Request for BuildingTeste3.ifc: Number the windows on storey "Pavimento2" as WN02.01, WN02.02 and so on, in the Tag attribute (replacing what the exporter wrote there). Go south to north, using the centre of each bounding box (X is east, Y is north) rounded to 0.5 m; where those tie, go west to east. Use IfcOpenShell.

First a look at what the model holds.

```python
import ifcopenshell
import ifcopenshell.util.element
import ifcopenshell.util.placement

model = ifcopenshell.open("BuildingTeste3.ifc")
print(model.schema)
storey = next(s for s in model.by_type("IfcBuildingStorey") if s.Name == "Pavimento2")
windows = [e for e in ifcopenshell.util.element.get_decomposition(storey) if e.is_a("IfcWindow")]
for e in sorted(windows, key=lambda e: e.id()):
    origin = ifcopenshell.util.placement.get_local_placement(e.ObjectPlacement)[:3, 3]
    print(e.id(), e.Tag, e.Name, origin.round(2) + 0.0, sep=" | ")
```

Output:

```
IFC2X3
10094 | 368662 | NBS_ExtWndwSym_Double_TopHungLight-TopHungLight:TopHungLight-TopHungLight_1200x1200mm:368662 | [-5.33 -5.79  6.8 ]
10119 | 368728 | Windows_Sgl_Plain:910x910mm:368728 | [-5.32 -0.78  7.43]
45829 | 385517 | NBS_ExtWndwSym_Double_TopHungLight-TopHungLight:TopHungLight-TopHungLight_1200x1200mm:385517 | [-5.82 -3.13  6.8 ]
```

```python
import ifcopenshell
import ifcopenshell.geom
import ifcopenshell.util.element
import ifcopenshell.util.shape

model = ifcopenshell.open("BuildingTeste3.ifc")
settings = ifcopenshell.geom.settings()
settings.set("use-world-coords", True)


def centre(element):
    shape = ifcopenshell.geom.create_shape(settings, element)
    return ifcopenshell.util.shape.get_bbox_centroid(shape.geometry)


storey = next(s for s in model.by_type("IfcBuildingStorey") if s.Name == "Pavimento2")
windows = [e for e in ifcopenshell.util.element.get_decomposition(storey) if e.is_a("IfcWindow")]

# Insertion points can sit at a corner or the storey origin, so sort by the geometry (in metres).
centres = {e: centre(e) for e in windows}
windows.sort(key=lambda e: (round(centres[e][1] / 0.5), centres[e][0]))

for i, e in enumerate(windows, start=1):
    number = f"WN02.{i:02d}"
    e.Tag = number
    print(e.id(), number)

model.write("BuildingTeste3_rev.ifc")
```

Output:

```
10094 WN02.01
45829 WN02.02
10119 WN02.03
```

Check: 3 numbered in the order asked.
